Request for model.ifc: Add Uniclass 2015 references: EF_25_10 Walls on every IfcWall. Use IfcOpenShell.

First a look at what the model holds.

```python
import ifcopenshell

model = ifcopenshell.open("model.ifc")
print(model.schema)
print("classifications:", [c.Name for c in model.by_type("IfcClassification")])
for ifc_class in ("IfcDoor", "IfcRoof", "IfcStair", "IfcWall", "IfcWindow"):
    print(ifc_class, len(model.by_type(ifc_class)))
```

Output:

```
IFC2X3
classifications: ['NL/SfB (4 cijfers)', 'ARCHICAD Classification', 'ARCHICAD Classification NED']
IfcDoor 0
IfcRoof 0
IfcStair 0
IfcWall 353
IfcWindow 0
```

```python
import ifcopenshell
import ifcopenshell.api.classification

model = ifcopenshell.open("model.ifc")

# IFC2X3 requires Source and Edition and has no link from the project to the system.
system = model.create_entity("IfcClassification", Source="NBS", Edition="2015", Name="Uniclass 2015")

codes = {
    "IfcWall": ("EF_25_10", "Walls"),
}
for ifc_class, (code, name) in codes.items():
    products = model.by_type(ifc_class)
    ifcopenshell.api.classification.add_reference(
        model, products=products, classification=system, identification=code, name=name
    )
    print(code, len(products))

model.write("model_rev.ifc")
```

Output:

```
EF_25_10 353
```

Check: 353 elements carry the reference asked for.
